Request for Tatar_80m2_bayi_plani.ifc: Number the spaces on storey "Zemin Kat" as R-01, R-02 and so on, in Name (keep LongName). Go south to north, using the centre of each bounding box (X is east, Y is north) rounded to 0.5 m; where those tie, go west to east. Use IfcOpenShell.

First a look at what the model holds.

```python
import ifcopenshell
import ifcopenshell.util.element
import ifcopenshell.util.placement

model = ifcopenshell.open("Tatar_80m2_bayi_plani.ifc")
print(model.schema)
storey = next(s for s in model.by_type("IfcBuildingStorey") if s.Name == "Zemin Kat")
spaces = [e for e in ifcopenshell.util.element.get_decomposition(storey) if e.is_a("IfcSpace")]
for e in sorted(spaces, key=lambda e: e.id()):
    origin = ifcopenshell.util.placement.get_local_placement(e.ObjectPlacement)[:3, 3]
    print(e.id(), e.Name, e.LongName, origin.round(2) + 0.0, sep=" | ")
```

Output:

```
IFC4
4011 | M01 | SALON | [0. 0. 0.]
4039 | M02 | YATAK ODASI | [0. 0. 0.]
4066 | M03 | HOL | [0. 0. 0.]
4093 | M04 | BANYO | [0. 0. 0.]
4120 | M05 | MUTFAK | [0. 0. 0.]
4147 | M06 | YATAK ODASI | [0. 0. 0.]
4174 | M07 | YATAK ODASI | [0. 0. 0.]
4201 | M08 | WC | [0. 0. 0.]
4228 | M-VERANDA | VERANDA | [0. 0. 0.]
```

```python
import ifcopenshell
import ifcopenshell.geom
import ifcopenshell.util.element
import ifcopenshell.util.shape

model = ifcopenshell.open("Tatar_80m2_bayi_plani.ifc")
settings = ifcopenshell.geom.settings()
settings.set("use-world-coords", True)


def centre(element):
    shape = ifcopenshell.geom.create_shape(settings, element)
    return ifcopenshell.util.shape.get_bbox_centroid(shape.geometry)


storey = next(s for s in model.by_type("IfcBuildingStorey") if s.Name == "Zemin Kat")
spaces = [e for e in ifcopenshell.util.element.get_decomposition(storey) if e.is_a("IfcSpace")]

# Insertion points can sit at a corner or the storey origin, so sort by the geometry (in metres).
centres = {e: centre(e) for e in spaces}
spaces.sort(key=lambda e: (round(centres[e][1] / 0.5), centres[e][0]))

for i, e in enumerate(spaces, start=1):
    number = f"R-{i:02d}"
    e.Name = number
    print(e.id(), number)

model.write("Tatar_80m2_bayi_plani_rev.ifc")
```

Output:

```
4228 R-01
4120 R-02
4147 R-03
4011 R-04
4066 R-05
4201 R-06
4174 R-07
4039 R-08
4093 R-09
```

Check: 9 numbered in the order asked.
